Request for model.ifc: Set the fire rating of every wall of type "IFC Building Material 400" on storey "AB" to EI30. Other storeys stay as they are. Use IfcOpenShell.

First a look at what the model holds.

```python
import ifcopenshell
import ifcopenshell.util.element

model = ifcopenshell.open("model.ifc")
print(model.schema)
storey = next(s for s in model.by_type("IfcBuildingStorey") if s.Name == "AB")
walls = [e for e in ifcopenshell.util.element.get_decomposition(storey) if e.is_a("IfcWall")]
seen = {}
for e in walls:
    element_type = ifcopenshell.util.element.get_type(e)
    key = (element_type.Name if element_type != e and element_type else None, ifcopenshell.util.element.get_pset(e, "Pset_WallCommon", "FireRating"))
    seen[key] = seen.get(key, 0) + 1
for (name, value), count in sorted(seen.items(), key=str):
    print(count, "x", name, "|", value)
```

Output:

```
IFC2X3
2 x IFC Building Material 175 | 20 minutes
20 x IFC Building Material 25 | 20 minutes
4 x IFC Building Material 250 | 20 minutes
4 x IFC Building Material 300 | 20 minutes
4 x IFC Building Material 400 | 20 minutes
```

```python
import ifcopenshell
import ifcopenshell.api.pset
import ifcopenshell.util.element

model = ifcopenshell.open("model.ifc")

storey = next(s for s in model.by_type("IfcBuildingStorey") if s.Name == "AB")
walls = [e for e in ifcopenshell.util.element.get_decomposition(storey) if e.is_a("IfcWall")]

count = 0
for e in walls:
    element_type = ifcopenshell.util.element.get_type(e)
    if element_type in (None, e) or element_type.Name != "IFC Building Material 400":
        continue
    # add_pset returns the element's existing set when there is one.
    pset = ifcopenshell.api.pset.add_pset(model, product=e, name="Pset_WallCommon")
    ifcopenshell.api.pset.edit_pset(model, pset=pset, properties={"FireRating": "EI30"})
    count += 1

print(count, "walls updated")

model.write("model_edited.ifc")
```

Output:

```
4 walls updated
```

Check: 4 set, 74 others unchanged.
